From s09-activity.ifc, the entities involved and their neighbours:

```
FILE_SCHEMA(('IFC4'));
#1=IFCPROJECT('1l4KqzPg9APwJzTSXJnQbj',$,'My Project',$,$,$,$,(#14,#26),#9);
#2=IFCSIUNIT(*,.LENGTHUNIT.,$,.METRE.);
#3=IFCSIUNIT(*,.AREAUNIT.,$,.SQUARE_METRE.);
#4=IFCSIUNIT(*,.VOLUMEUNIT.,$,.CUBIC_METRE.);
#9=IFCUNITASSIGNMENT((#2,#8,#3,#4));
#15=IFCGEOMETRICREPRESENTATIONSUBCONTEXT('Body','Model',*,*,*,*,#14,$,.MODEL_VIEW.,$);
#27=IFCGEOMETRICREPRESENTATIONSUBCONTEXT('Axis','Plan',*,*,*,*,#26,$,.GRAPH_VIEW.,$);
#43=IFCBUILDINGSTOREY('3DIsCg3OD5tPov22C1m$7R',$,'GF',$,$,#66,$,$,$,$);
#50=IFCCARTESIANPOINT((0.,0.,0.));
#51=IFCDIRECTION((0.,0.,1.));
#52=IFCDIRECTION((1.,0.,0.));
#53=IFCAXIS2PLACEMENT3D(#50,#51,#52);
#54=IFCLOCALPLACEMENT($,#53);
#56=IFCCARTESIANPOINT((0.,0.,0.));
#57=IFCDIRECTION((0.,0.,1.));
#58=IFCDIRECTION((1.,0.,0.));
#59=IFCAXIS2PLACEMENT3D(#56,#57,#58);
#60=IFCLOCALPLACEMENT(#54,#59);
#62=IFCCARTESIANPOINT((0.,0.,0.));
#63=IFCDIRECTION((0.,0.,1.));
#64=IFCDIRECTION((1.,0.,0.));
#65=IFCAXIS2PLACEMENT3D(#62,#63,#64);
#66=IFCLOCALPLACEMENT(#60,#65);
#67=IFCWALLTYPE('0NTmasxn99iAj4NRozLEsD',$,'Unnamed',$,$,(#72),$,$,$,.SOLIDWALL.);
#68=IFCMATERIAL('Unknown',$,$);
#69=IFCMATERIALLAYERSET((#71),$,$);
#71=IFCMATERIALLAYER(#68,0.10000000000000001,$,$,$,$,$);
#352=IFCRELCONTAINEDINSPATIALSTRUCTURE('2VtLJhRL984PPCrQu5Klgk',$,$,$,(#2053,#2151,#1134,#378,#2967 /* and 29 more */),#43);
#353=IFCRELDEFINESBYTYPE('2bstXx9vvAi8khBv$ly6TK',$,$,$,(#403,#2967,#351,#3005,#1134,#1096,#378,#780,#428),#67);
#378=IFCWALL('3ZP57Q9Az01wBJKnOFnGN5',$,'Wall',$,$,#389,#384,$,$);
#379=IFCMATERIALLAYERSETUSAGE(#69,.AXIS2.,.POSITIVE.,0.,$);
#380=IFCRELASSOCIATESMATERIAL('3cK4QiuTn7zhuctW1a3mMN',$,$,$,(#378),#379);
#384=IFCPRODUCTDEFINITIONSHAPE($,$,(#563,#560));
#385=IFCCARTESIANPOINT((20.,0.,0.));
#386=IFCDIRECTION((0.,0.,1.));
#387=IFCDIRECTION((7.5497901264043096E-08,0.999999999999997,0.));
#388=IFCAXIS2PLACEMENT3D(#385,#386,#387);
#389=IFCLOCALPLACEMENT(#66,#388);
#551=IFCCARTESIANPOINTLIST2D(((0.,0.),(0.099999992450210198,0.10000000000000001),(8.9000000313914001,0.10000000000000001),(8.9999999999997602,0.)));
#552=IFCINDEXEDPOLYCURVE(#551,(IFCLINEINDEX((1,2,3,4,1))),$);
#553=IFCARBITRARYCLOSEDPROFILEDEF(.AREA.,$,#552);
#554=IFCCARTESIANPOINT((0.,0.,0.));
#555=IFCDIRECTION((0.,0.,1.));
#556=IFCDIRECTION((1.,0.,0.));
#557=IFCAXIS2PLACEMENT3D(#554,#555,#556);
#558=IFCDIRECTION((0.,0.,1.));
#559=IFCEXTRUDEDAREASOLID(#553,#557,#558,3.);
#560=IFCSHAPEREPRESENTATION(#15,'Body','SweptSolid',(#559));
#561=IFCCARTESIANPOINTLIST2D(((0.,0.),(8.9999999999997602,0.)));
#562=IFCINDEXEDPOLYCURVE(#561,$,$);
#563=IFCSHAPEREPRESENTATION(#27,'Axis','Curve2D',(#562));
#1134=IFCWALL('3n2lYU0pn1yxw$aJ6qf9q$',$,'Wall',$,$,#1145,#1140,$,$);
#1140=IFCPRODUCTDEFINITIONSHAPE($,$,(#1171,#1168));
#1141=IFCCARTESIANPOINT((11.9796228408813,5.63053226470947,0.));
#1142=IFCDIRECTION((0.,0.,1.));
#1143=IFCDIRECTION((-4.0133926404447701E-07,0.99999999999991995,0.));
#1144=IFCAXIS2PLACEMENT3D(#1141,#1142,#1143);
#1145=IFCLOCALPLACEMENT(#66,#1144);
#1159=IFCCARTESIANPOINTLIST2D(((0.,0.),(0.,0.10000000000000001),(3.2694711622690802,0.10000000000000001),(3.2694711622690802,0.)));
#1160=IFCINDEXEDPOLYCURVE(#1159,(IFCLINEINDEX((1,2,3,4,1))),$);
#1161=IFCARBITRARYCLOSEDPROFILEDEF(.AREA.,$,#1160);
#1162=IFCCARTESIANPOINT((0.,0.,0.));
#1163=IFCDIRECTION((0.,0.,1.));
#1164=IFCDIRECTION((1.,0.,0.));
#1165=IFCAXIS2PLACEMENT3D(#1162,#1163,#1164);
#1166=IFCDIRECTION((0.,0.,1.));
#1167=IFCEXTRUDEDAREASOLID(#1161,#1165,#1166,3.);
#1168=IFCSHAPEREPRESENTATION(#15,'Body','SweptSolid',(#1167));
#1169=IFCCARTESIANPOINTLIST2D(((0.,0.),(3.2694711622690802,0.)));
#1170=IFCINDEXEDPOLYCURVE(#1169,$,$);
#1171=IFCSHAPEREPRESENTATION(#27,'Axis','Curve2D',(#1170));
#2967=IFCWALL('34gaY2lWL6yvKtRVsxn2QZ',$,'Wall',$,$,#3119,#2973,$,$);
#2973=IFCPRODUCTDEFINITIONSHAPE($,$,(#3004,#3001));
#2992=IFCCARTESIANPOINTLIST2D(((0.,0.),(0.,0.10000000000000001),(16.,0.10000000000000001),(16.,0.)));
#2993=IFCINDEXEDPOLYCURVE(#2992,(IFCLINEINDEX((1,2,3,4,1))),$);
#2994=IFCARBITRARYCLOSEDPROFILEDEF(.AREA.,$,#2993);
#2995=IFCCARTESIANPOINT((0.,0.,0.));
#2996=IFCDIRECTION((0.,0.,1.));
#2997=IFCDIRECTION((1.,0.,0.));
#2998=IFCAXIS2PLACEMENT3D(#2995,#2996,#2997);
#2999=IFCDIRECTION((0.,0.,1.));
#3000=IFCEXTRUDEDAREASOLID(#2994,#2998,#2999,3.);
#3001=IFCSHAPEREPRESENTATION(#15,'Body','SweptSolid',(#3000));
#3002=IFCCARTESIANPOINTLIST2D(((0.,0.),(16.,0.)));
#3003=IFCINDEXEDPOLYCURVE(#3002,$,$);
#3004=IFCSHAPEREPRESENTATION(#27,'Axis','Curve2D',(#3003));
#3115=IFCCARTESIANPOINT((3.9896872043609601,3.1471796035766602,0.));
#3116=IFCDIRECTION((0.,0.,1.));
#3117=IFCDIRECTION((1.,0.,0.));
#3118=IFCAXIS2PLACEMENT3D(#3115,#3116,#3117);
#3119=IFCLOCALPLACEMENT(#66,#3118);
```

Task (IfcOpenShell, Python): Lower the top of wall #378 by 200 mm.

```python
import ifcopenshell
import ifcopenshell.geom
import ifcopenshell.util.representation
import ifcopenshell.util.shape
import ifcopenshell.util.unit

model = ifcopenshell.open("s09-activity.ifc")
unit_scale = ifcopenshell.util.unit.calculate_unit_scale(model)
settings = ifcopenshell.geom.settings()


def volume(element):
    """Net volume in cubic metres, openings subtracted."""
    shape = ifcopenshell.geom.create_shape(settings, element)
    return ifcopenshell.util.shape.get_volume(shape.geometry)


wall = model.by_id(378)
before = volume(wall)

body = ifcopenshell.util.representation.get_representation(wall, "Model", "Body")
solid = body.Items[0]
old_height = solid.Depth
solid.Depth -= 0.2 / unit_scale
after = volume(wall)

print(f"height {old_height:g} -> {solid.Depth:g}, volume {before:.3f} -> {after:.3f} m3")

model.write("s09-activity_updated.ifc")
```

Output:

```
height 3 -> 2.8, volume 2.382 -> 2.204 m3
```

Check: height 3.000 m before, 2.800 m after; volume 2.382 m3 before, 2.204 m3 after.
